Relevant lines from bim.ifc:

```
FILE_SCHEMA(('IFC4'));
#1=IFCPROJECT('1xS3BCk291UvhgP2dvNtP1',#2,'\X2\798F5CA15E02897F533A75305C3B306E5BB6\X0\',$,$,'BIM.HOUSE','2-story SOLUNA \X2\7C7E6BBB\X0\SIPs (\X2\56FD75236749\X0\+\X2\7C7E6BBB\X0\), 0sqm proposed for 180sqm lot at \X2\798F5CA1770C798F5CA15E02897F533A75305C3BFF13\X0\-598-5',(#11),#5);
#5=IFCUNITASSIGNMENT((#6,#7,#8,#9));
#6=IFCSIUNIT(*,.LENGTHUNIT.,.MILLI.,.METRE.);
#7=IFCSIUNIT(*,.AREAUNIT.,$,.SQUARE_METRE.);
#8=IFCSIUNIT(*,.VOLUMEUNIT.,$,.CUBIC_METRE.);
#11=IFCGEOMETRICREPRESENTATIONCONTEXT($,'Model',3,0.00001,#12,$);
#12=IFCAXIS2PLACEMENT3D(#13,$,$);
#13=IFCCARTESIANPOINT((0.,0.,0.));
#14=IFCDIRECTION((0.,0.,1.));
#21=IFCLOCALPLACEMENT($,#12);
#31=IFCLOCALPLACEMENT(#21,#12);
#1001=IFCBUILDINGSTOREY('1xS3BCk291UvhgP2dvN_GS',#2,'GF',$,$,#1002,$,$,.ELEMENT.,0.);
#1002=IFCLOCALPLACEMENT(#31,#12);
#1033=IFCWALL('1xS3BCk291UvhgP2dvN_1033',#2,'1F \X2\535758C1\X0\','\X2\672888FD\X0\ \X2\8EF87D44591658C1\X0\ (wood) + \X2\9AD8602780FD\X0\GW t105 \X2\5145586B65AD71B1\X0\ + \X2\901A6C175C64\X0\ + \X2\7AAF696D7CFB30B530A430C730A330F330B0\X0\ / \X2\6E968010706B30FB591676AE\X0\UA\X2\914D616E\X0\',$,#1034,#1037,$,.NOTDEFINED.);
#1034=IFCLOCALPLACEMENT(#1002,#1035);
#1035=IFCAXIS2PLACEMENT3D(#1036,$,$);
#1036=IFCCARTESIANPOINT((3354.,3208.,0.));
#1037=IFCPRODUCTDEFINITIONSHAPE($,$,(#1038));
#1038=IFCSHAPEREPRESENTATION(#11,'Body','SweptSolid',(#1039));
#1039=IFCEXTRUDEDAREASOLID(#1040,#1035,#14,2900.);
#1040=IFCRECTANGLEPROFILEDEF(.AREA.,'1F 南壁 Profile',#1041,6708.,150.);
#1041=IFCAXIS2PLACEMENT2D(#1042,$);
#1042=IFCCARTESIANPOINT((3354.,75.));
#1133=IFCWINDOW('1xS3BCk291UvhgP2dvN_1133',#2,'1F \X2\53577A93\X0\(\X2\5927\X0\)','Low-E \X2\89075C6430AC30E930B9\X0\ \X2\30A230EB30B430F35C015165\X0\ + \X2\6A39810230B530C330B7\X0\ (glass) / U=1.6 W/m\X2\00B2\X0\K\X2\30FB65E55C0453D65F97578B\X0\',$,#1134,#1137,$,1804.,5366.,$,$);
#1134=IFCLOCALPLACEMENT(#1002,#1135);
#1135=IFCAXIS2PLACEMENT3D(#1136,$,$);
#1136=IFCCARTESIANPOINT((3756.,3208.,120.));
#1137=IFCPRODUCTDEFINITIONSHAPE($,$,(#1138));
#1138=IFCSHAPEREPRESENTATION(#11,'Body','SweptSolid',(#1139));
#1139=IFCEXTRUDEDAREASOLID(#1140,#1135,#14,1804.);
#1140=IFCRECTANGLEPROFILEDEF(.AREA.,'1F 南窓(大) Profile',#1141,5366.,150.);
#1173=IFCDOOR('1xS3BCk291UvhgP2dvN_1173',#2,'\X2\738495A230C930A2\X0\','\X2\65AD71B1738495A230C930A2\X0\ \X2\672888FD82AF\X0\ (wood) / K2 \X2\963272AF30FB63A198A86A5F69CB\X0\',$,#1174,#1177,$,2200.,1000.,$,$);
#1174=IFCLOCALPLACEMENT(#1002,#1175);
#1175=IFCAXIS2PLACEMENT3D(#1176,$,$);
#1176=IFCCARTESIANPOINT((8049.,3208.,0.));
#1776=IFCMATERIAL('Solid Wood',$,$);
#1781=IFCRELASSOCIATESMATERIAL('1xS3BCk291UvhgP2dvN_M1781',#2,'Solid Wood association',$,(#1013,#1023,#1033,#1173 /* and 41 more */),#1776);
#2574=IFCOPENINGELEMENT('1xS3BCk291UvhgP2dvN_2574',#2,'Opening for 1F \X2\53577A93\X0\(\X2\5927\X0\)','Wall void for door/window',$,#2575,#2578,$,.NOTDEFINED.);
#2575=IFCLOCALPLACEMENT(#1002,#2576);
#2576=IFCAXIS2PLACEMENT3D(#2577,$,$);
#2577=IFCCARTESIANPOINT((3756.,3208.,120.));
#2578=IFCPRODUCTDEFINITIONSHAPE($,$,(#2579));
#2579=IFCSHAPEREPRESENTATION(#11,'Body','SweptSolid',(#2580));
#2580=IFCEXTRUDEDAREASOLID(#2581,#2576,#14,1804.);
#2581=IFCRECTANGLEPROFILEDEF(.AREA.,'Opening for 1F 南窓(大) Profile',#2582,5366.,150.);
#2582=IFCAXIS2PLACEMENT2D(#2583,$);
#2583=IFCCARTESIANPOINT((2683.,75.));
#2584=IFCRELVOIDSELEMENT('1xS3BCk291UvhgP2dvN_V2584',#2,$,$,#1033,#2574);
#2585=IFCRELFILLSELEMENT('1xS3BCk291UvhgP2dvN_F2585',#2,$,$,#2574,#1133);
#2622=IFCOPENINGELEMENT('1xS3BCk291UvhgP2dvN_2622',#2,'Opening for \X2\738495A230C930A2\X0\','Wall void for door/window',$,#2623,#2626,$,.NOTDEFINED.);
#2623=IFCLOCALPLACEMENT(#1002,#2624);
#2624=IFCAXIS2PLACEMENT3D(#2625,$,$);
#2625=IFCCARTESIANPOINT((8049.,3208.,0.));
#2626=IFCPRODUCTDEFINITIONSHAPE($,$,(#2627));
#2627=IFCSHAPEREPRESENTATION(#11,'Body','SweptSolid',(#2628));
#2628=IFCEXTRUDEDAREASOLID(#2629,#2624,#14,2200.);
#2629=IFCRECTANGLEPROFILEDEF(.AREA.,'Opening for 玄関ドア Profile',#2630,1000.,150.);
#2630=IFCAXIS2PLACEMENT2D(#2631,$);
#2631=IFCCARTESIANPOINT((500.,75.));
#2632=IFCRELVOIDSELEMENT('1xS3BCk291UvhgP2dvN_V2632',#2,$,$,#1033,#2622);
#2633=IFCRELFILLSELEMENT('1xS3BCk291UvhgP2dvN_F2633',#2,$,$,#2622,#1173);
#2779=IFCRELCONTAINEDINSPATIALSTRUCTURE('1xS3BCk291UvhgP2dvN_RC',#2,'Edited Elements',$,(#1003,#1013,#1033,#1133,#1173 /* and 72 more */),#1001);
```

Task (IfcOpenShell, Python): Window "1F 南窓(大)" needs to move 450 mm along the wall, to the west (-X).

```python
import ifcopenshell
import ifcopenshell.api.geometry
import ifcopenshell.util.placement

model = ifcopenshell.open("bim.ifc")

window = model.by_id(1133)
opening = window.FillsVoids[0].RelatingOpeningElement
wall = opening.VoidsElements[0].RelatingBuildingElement

wall_matrix = ifcopenshell.util.placement.get_local_placement(wall.ObjectPlacement)
shift = wall_matrix[:3, 0] * -450.0
before = ifcopenshell.util.placement.get_local_placement(window.ObjectPlacement)[:3, 3].copy()

# The window is not placed relative to its opening, so move both.
for product in (opening, window):
    matrix = ifcopenshell.util.placement.get_local_placement(product.ObjectPlacement)
    matrix[:3, 3] += shift
    ifcopenshell.api.geometry.edit_object_placement(model, product=product, matrix=matrix, is_si=False)

after = ifcopenshell.util.placement.get_local_placement(window.ObjectPlacement)[:3, 3]
print("window moved by", (after - before).round(3) + 0.0)

model.write("bim_edited.ifc")
```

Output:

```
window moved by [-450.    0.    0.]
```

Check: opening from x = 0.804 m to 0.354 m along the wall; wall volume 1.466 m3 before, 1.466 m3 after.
